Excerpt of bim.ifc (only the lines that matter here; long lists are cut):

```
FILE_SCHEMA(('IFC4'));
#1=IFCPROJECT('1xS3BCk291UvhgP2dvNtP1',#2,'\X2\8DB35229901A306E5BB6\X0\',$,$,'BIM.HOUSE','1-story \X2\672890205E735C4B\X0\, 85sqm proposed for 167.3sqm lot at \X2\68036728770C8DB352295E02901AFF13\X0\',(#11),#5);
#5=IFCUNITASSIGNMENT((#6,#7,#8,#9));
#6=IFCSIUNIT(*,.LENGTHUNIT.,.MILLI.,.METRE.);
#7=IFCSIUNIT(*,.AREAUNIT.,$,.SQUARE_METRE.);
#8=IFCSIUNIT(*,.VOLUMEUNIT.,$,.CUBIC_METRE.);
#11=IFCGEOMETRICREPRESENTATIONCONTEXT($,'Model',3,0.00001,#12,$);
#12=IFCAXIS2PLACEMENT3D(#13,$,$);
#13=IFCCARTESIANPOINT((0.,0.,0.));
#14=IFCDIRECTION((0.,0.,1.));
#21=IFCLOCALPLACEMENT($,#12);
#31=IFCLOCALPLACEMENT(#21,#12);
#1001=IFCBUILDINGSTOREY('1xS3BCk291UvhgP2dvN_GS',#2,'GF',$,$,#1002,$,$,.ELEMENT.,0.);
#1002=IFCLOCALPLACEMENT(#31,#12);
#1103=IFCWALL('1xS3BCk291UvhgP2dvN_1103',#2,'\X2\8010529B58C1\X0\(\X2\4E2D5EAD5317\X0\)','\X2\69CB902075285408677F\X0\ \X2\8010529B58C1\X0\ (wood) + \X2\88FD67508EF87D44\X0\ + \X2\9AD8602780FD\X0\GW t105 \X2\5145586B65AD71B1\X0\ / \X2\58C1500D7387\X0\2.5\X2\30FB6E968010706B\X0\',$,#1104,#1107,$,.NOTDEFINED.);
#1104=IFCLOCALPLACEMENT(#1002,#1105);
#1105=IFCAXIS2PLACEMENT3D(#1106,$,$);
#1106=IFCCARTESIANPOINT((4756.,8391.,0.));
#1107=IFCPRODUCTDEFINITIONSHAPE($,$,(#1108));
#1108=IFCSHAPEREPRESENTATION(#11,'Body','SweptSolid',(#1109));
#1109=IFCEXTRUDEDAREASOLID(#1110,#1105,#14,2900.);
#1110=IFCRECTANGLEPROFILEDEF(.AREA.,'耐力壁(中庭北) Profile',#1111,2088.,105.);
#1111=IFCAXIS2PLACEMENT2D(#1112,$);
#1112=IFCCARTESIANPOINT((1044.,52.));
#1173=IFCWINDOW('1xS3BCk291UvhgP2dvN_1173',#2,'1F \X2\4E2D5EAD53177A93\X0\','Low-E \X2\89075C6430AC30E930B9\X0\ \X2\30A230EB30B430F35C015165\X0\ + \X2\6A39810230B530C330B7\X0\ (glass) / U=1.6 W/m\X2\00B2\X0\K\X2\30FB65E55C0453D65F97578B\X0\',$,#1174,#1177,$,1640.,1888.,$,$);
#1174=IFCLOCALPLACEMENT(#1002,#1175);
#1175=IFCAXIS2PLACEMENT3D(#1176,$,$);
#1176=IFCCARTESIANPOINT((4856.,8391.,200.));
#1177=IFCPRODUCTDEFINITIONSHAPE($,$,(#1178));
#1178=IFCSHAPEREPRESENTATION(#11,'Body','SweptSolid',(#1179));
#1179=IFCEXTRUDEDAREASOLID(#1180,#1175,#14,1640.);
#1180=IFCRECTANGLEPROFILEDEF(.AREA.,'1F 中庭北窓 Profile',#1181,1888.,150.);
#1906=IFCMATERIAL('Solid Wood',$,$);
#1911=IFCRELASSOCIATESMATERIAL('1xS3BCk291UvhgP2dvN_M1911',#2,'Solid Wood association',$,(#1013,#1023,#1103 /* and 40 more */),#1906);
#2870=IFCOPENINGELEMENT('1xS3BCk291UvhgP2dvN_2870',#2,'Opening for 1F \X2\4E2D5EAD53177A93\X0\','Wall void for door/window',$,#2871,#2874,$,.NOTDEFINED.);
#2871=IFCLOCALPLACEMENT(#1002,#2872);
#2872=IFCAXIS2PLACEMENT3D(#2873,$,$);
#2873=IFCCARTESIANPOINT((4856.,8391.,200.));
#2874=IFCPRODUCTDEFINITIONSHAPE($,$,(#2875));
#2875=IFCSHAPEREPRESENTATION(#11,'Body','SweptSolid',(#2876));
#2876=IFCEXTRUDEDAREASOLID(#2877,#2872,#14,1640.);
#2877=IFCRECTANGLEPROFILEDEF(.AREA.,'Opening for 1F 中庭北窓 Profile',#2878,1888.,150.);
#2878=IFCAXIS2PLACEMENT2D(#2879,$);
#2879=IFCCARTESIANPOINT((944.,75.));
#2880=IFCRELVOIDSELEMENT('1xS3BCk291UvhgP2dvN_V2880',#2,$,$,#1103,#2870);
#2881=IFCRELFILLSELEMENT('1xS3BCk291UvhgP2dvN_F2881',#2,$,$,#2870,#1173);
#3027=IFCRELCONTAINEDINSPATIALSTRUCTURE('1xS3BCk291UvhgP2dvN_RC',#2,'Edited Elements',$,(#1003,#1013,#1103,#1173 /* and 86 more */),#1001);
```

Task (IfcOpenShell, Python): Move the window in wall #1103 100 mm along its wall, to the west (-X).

```python
import ifcopenshell
import ifcopenshell.api.geometry
import ifcopenshell.util.placement

model = ifcopenshell.open("bim.ifc")

window = model.by_guid("1xS3BCk291UvhgP2dvN_1173")
opening = window.FillsVoids[0].RelatingOpeningElement
wall = opening.VoidsElements[0].RelatingBuildingElement

wall_matrix = ifcopenshell.util.placement.get_local_placement(wall.ObjectPlacement)
shift = wall_matrix[:3, 0] * -100.0
before = ifcopenshell.util.placement.get_local_placement(window.ObjectPlacement)[:3, 3].copy()

# The window is not placed relative to its opening, so move both.
for product in (opening, window):
    matrix = ifcopenshell.util.placement.get_local_placement(product.ObjectPlacement)
    matrix[:3, 3] += shift
    ifcopenshell.api.geometry.edit_object_placement(model, product=product, matrix=matrix, is_si=False)

after = ifcopenshell.util.placement.get_local_placement(window.ObjectPlacement)[:3, 3]
print("window moved by", (after - before).round(3) + 0.0)

model.write("bim_rev.ifc")
```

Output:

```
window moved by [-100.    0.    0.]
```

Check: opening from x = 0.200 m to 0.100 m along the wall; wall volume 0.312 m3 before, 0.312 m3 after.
